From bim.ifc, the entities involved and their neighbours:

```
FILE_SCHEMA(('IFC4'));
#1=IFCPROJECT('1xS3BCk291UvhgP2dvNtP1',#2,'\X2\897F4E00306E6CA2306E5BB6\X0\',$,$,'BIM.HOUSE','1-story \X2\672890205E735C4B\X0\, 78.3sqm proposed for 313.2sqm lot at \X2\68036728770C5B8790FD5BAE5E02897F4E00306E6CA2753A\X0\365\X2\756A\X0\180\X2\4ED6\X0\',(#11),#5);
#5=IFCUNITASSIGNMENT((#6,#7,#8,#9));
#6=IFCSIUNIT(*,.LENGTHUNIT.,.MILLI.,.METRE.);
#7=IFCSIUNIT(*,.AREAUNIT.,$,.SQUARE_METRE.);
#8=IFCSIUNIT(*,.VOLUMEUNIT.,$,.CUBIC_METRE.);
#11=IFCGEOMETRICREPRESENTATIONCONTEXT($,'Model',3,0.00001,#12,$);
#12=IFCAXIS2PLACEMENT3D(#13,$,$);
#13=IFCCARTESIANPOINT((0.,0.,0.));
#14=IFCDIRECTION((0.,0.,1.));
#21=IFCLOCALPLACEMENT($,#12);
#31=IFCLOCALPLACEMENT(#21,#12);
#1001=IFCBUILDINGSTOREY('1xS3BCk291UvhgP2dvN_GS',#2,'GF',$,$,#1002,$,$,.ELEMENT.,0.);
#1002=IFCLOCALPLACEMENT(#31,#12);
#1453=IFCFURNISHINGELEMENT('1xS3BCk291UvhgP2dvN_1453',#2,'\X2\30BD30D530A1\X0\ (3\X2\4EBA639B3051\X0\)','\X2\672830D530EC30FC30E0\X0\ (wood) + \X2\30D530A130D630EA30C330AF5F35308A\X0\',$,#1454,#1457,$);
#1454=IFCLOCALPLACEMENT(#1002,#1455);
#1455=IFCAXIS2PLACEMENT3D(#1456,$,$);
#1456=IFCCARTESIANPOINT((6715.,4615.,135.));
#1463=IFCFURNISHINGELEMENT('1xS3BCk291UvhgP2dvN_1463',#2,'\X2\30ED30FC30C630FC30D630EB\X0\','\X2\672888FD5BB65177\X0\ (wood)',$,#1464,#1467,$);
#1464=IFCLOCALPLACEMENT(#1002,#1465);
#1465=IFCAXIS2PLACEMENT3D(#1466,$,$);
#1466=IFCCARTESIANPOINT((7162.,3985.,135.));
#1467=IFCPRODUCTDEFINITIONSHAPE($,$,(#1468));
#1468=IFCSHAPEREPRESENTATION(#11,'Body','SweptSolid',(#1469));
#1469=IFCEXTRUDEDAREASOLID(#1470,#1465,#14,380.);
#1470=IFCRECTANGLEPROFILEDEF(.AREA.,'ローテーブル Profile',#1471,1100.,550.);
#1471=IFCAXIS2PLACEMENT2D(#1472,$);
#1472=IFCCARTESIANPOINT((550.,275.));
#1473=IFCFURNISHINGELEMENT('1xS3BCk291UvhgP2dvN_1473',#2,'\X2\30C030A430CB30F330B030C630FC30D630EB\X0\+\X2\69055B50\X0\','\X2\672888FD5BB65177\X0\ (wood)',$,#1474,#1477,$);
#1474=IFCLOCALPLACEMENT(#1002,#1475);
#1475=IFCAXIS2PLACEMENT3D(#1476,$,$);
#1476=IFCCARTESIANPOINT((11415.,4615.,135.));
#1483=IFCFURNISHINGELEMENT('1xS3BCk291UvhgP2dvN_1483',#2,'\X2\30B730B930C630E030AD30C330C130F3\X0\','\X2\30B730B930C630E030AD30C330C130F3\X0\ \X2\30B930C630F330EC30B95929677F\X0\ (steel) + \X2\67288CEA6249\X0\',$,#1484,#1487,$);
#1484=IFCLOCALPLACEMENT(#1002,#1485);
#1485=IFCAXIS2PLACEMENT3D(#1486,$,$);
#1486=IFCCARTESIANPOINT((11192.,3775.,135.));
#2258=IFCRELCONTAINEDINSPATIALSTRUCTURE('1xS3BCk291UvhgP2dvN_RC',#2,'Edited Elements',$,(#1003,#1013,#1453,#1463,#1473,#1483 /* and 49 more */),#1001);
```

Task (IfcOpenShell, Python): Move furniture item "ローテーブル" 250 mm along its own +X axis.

```python
import ifcopenshell
import ifcopenshell.api.geometry
import ifcopenshell.util.placement
import ifcopenshell.util.unit

model = ifcopenshell.open("bim.ifc")
unit_scale = ifcopenshell.util.unit.calculate_unit_scale(model)

item = model.by_id(1463)
matrix = ifcopenshell.util.placement.get_local_placement(item.ObjectPlacement)
matrix[:3, 3] += matrix[:3, 0] * 0.25 / unit_scale
ifcopenshell.api.geometry.edit_object_placement(model, product=item, matrix=matrix, is_si=False)

print(ifcopenshell.util.placement.get_local_placement(item.ObjectPlacement).round(3) + 0.0)

model.write("bim_v2.ifc")
```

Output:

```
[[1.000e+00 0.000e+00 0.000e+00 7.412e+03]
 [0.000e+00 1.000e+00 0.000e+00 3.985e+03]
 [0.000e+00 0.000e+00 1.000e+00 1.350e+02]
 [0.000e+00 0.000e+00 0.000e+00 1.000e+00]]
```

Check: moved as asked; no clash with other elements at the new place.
